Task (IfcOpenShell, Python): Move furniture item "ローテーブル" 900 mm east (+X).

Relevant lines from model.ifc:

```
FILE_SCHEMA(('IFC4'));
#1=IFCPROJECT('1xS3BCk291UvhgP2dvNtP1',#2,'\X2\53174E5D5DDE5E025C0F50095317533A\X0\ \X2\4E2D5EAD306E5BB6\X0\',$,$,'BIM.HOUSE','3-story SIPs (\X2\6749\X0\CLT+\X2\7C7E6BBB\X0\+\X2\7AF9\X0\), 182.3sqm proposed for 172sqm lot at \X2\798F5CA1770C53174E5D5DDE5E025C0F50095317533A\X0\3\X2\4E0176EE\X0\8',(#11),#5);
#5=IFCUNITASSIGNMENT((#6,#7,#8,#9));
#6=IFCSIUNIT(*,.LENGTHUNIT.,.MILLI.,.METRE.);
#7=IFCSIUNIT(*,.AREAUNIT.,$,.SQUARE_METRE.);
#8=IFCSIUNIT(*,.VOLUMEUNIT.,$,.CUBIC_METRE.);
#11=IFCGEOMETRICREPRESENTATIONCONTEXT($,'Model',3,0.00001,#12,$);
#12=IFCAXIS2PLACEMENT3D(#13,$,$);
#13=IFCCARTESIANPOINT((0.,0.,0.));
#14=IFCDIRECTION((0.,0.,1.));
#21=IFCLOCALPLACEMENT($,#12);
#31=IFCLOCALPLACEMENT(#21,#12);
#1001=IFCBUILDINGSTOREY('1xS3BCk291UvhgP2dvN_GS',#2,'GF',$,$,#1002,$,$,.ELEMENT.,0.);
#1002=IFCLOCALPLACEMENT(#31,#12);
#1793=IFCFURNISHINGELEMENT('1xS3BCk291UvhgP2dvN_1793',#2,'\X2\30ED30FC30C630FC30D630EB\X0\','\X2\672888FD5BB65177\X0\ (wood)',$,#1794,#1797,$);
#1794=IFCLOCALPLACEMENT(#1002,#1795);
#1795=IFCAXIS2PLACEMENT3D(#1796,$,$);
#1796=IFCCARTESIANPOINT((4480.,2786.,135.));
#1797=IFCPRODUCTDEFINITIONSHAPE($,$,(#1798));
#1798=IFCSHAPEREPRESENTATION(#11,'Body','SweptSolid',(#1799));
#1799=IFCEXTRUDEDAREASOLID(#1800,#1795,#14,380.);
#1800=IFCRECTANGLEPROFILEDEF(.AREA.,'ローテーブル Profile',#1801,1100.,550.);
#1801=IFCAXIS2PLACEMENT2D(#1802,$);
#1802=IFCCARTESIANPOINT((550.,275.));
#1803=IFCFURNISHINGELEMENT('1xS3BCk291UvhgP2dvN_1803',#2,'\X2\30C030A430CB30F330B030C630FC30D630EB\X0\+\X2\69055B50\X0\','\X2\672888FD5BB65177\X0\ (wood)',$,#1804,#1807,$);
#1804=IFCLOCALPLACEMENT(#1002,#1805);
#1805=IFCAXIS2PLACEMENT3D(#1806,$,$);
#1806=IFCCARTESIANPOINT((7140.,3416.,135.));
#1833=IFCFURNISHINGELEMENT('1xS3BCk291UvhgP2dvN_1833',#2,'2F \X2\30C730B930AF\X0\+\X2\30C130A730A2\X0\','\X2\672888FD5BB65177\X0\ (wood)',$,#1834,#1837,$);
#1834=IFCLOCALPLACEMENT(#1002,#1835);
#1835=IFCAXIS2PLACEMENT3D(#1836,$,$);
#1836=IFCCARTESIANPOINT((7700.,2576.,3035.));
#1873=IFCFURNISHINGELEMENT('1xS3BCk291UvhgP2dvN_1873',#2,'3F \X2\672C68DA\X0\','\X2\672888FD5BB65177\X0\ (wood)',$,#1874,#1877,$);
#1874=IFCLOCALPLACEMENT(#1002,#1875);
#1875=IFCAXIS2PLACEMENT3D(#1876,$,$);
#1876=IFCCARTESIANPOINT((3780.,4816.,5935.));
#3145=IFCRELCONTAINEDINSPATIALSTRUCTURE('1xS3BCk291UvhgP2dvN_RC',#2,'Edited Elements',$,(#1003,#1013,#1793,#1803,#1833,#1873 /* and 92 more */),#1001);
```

```python
import ifcopenshell
import ifcopenshell.api.geometry
import ifcopenshell.util.placement
import ifcopenshell.util.unit

model = ifcopenshell.open("model.ifc")
unit_scale = ifcopenshell.util.unit.calculate_unit_scale(model)

item = model.by_id(1793)
matrix = ifcopenshell.util.placement.get_local_placement(item.ObjectPlacement)
matrix[0, 3] += 0.9 / unit_scale
ifcopenshell.api.geometry.edit_object_placement(model, product=item, matrix=matrix, is_si=False)

print(ifcopenshell.util.placement.get_local_placement(item.ObjectPlacement).round(3) + 0.0)

model.write("model_rev.ifc")
```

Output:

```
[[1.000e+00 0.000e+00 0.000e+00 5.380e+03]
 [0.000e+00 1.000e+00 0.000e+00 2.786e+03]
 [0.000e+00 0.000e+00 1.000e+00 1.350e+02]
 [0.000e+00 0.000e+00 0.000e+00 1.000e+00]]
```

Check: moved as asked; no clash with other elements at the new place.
